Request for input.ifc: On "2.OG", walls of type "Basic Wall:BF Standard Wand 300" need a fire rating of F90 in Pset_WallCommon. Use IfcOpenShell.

First a look at what the model holds.

```python
import ifcopenshell
import ifcopenshell.util.element

model = ifcopenshell.open("input.ifc")
print(model.schema)
storey = next(s for s in model.by_type("IfcBuildingStorey") if s.Name == "2.OG")
walls = [e for e in ifcopenshell.util.element.get_decomposition(storey) if e.is_a("IfcWall")]
seen = {}
for e in walls:
    element_type = ifcopenshell.util.element.get_type(e)
    key = (element_type.Name if element_type != e and element_type else None, ifcopenshell.util.element.get_pset(e, "Pset_WallCommon", "FireRating"))
    seen[key] = seen.get(key, 0) + 1
for (name, value), count in sorted(seen.items(), key=str):
    print(count, "x", name, "|", value)
```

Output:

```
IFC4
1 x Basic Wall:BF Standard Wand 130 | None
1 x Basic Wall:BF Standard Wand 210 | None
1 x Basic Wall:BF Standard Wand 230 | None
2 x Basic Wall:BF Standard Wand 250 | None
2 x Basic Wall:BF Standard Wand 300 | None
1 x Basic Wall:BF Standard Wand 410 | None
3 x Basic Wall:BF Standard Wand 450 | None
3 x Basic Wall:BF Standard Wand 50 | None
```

```python
import ifcopenshell
import ifcopenshell.api.pset
import ifcopenshell.util.element

model = ifcopenshell.open("input.ifc")

storey = next(s for s in model.by_type("IfcBuildingStorey") if s.Name == "2.OG")
walls = [e for e in ifcopenshell.util.element.get_decomposition(storey) if e.is_a("IfcWall")]

count = 0
for e in walls:
    element_type = ifcopenshell.util.element.get_type(e)
    if element_type in (None, e) or element_type.Name != "Basic Wall:BF Standard Wand 300":
        continue
    # add_pset returns the element's existing set when there is one.
    pset = ifcopenshell.api.pset.add_pset(model, product=e, name="Pset_WallCommon")
    ifcopenshell.api.pset.edit_pset(model, pset=pset, properties={"FireRating": "F90"})
    count += 1

print(count, "walls updated")

model.write("input_updated.ifc")
```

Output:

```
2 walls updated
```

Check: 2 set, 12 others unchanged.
